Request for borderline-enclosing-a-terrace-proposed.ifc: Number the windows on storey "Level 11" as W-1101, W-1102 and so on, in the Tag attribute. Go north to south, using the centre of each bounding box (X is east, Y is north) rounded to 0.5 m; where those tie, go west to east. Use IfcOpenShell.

First a look at what the model holds.

```python
import ifcopenshell
import ifcopenshell.util.element
import ifcopenshell.util.placement

model = ifcopenshell.open("borderline-enclosing-a-terrace-proposed.ifc")
print(model.schema)
storey = next(s for s in model.by_type("IfcBuildingStorey") if s.Name == "Level 11")
windows = [e for e in ifcopenshell.util.element.get_decomposition(storey) if e.is_a("IfcWindow")]
for e in sorted(windows, key=lambda e: e.id()):
    origin = ifcopenshell.util.placement.get_local_placement(e.ObjectPlacement)[:3, 3]
    print(e.id(), e.Tag, e.Name, origin.round(2) + 0.0, sep=" | ")
```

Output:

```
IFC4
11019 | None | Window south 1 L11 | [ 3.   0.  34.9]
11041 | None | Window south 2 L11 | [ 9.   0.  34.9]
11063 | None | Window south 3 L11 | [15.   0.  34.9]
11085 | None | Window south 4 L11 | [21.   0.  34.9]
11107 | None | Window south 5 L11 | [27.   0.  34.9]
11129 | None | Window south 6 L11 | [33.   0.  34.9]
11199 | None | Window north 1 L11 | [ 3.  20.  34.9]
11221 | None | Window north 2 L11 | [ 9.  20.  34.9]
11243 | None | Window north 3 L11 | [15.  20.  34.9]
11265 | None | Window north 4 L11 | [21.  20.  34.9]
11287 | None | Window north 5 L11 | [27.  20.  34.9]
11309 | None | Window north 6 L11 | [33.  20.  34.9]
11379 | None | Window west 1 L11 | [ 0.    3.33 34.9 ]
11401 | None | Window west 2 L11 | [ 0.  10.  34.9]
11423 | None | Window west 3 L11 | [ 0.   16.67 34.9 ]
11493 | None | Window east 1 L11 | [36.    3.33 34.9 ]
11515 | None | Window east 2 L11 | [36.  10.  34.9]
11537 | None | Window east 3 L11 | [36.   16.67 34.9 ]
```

```python
import ifcopenshell
import ifcopenshell.geom
import ifcopenshell.util.element
import ifcopenshell.util.shape

model = ifcopenshell.open("borderline-enclosing-a-terrace-proposed.ifc")
settings = ifcopenshell.geom.settings()
settings.set("use-world-coords", True)


def centre(element):
    shape = ifcopenshell.geom.create_shape(settings, element)
    return ifcopenshell.util.shape.get_bbox_centroid(shape.geometry)


storey = next(s for s in model.by_type("IfcBuildingStorey") if s.Name == "Level 11")
windows = [e for e in ifcopenshell.util.element.get_decomposition(storey) if e.is_a("IfcWindow")]

# Insertion points can sit at a corner or the storey origin, so sort by the geometry (in metres).
centres = {e: centre(e) for e in windows}
windows.sort(key=lambda e: (-round(centres[e][1] / 0.5), centres[e][0]))

for i, e in enumerate(windows, start=1):
    number = f"W-11{i:02d}"
    e.Tag = number
    print(e.id(), number)

model.write("borderline-enclosing-a-terrace-proposed-out.ifc")
```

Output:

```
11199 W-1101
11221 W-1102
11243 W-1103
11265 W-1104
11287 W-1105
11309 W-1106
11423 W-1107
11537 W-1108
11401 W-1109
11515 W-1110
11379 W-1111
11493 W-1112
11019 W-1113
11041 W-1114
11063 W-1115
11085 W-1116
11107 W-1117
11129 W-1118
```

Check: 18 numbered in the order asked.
